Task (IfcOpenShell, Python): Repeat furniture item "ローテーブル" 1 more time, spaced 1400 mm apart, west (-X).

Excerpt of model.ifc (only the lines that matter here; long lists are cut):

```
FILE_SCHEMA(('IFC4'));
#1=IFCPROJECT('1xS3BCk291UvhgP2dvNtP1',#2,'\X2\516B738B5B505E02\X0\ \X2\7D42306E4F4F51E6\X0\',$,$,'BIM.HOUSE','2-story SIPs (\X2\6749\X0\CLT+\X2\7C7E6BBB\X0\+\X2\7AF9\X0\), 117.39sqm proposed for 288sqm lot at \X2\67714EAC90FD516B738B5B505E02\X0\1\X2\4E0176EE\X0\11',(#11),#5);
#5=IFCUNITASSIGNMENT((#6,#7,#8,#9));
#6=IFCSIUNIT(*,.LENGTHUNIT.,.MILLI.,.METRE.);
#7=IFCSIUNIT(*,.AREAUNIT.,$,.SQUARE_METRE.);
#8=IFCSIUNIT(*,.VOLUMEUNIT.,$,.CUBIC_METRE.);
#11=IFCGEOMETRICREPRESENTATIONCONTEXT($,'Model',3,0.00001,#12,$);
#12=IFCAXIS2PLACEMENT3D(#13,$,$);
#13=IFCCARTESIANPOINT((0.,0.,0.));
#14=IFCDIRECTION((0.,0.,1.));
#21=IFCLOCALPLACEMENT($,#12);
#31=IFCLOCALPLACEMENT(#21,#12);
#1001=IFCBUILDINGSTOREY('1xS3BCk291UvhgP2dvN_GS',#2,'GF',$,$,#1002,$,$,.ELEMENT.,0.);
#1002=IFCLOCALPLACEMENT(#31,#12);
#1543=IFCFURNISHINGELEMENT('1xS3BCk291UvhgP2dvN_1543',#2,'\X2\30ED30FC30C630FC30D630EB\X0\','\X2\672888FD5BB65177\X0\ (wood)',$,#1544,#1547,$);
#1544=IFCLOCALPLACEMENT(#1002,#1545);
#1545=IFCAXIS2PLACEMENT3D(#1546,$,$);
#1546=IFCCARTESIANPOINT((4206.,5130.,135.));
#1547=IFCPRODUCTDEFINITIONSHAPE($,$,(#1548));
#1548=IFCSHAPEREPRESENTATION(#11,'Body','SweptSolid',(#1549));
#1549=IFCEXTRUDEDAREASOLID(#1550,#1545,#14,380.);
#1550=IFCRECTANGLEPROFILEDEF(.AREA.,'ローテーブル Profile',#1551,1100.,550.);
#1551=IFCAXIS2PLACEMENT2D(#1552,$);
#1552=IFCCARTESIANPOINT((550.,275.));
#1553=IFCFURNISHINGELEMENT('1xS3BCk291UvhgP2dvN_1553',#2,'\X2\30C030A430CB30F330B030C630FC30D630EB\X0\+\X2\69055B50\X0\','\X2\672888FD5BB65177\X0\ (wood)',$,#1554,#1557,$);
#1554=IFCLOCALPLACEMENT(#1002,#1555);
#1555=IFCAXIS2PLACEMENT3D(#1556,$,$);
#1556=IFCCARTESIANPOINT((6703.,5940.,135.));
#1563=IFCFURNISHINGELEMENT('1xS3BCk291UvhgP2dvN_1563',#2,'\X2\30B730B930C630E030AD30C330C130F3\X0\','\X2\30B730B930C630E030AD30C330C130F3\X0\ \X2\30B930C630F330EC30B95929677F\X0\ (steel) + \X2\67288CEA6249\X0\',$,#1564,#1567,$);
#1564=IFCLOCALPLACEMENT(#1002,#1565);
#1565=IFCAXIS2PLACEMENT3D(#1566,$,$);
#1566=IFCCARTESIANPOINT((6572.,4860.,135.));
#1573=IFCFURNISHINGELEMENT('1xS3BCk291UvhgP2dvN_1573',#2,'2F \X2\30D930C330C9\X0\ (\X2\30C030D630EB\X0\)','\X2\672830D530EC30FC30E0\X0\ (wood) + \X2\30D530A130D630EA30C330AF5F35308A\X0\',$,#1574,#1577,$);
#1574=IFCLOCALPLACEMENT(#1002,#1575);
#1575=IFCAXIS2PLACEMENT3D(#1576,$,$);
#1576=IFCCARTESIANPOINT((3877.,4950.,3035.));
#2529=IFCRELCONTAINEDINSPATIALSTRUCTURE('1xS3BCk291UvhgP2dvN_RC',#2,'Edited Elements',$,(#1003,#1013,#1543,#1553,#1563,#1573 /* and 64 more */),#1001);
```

```python
import numpy as np
import ifcopenshell
import ifcopenshell.api.geometry
import ifcopenshell.api.root
import ifcopenshell.util.element
import ifcopenshell.util.placement
import ifcopenshell.util.unit

model = ifcopenshell.open("model.ifc")
unit_scale = ifcopenshell.util.unit.calculate_unit_scale(model)


def reuse_history(source, copy):
    """copy_class also copies each property set's owner history, people and application; keep the originals."""
    for rel in copy.IsDefinedBy:
        if rel.is_a("IfcRelDefinesByProperties") and (history := rel.RelatingPropertyDefinition.OwnerHistory):
            rel.RelatingPropertyDefinition.OwnerHistory = source.OwnerHistory
            ifcopenshell.util.element.remove_deep2(model, history)


source = model.by_id(1543)
base = ifcopenshell.util.placement.get_local_placement(source.ObjectPlacement)
step = np.array([-1.0, 0.0, 0.0]) * 1.4 / unit_scale

for i in range(1, 2):
    copy = ifcopenshell.api.root.copy_class(model, product=source)
    copy.Representation = ifcopenshell.util.element.copy_deep(
        model, source.Representation, exclude=["IfcGeometricRepresentationContext", "IfcRepresentationMap"]
    )
    reuse_history(source, copy)
    matrix = base.copy()
    matrix[:3, 3] += i * step
    print("added at", matrix[:3, 3].round(3) + 0.0)
    ifcopenshell.api.geometry.edit_object_placement(model, product=copy, matrix=matrix, is_si=False)

model.write("model_edited.ifc")
```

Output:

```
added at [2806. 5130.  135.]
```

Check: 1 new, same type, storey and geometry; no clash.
